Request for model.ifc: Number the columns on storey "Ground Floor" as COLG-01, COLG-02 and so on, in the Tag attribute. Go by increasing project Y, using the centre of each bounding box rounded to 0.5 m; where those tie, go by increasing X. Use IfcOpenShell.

First a look at what the model holds.

```python
import ifcopenshell
import ifcopenshell.util.element
import ifcopenshell.util.placement

model = ifcopenshell.open("model.ifc")
print(model.schema)
storey = next(s for s in model.by_type("IfcBuildingStorey") if s.Name == "Ground Floor")
columns = [e for e in ifcopenshell.util.element.get_decomposition(storey) if e.is_a("IfcColumn")]
for e in sorted(columns, key=lambda e: e.id()):
    origin = ifcopenshell.util.placement.get_local_placement(e.ObjectPlacement)[:3, 3]
    print(e.id(), e.Tag, e.Name, origin.round(2) + 0.0, sep=" | ")
```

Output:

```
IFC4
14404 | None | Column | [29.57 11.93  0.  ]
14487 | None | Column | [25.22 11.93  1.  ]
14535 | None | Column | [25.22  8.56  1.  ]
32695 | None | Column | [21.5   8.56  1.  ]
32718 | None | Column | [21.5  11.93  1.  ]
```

```python
import ifcopenshell
import ifcopenshell.geom
import ifcopenshell.util.element
import ifcopenshell.util.shape

model = ifcopenshell.open("model.ifc")
settings = ifcopenshell.geom.settings()
settings.set("use-world-coords", True)


def centre(element):
    shape = ifcopenshell.geom.create_shape(settings, element)
    return ifcopenshell.util.shape.get_bbox_centroid(shape.geometry)


storey = next(s for s in model.by_type("IfcBuildingStorey") if s.Name == "Ground Floor")
columns = [e for e in ifcopenshell.util.element.get_decomposition(storey) if e.is_a("IfcColumn")]

# Insertion points can sit at a corner or the storey origin, so sort by the geometry (in metres).
centres = {e: centre(e) for e in columns}
columns.sort(key=lambda e: (round(centres[e][1] / 0.5), centres[e][0]))

for i, e in enumerate(columns, start=1):
    number = f"COLG-{i:02d}"
    e.Tag = number
    print(e.id(), number)

model.write("model_rev.ifc")
```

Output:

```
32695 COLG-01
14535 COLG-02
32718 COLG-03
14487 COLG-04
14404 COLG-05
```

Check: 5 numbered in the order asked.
